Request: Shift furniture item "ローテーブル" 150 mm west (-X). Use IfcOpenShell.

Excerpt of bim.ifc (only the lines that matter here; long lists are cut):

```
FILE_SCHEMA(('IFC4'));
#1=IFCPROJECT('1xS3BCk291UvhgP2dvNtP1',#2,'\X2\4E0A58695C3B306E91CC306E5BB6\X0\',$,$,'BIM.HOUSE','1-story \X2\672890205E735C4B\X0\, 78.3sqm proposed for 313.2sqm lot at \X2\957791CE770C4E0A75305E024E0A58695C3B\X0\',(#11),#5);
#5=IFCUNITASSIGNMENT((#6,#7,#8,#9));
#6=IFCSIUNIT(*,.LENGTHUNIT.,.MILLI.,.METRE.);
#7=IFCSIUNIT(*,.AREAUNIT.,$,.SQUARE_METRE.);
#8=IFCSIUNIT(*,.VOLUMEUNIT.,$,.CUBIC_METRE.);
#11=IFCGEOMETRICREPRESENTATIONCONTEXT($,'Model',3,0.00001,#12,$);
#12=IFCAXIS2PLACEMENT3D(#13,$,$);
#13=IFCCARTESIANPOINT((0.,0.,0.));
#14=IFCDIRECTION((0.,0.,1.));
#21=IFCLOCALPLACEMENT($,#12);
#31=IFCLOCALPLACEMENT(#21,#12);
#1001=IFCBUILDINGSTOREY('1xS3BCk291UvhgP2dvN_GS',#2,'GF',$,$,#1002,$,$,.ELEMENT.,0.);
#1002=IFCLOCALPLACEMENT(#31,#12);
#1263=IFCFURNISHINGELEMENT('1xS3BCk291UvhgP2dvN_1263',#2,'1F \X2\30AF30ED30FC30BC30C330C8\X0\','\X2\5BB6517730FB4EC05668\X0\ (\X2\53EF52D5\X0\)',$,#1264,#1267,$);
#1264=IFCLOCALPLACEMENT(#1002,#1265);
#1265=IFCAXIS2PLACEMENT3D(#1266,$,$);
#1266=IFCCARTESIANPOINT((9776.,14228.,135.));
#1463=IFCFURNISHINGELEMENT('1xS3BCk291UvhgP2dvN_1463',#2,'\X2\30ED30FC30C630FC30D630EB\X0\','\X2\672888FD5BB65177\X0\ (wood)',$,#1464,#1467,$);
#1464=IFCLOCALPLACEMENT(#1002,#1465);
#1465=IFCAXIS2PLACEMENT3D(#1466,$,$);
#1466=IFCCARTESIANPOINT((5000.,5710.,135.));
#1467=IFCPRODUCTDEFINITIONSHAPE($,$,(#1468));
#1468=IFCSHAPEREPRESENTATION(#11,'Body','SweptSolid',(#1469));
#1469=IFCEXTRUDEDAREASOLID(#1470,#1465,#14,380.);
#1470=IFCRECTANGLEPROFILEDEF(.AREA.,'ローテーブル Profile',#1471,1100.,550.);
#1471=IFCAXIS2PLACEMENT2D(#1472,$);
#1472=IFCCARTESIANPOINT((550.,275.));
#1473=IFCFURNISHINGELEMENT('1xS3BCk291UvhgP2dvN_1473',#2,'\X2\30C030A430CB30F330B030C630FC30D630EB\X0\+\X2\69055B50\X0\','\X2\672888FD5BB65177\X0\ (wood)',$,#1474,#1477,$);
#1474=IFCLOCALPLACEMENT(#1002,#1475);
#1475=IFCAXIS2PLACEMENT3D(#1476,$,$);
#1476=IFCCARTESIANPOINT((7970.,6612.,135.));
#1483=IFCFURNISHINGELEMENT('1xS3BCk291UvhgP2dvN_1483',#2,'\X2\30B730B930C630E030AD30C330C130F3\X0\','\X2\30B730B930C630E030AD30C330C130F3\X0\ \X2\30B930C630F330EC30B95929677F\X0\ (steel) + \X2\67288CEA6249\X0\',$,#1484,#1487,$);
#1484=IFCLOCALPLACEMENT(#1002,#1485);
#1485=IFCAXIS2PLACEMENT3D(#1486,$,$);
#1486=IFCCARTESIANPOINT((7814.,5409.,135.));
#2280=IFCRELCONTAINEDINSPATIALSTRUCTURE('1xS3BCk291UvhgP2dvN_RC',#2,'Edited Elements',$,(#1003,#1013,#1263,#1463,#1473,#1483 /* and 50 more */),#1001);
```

```python
import ifcopenshell
import ifcopenshell.api.geometry
import ifcopenshell.util.placement
import ifcopenshell.util.unit

model = ifcopenshell.open("bim.ifc")
unit_scale = ifcopenshell.util.unit.calculate_unit_scale(model)

item = model.by_id(1463)
matrix = ifcopenshell.util.placement.get_local_placement(item.ObjectPlacement)
matrix[0, 3] -= 0.15 / unit_scale
ifcopenshell.api.geometry.edit_object_placement(model, product=item, matrix=matrix, is_si=False)

print(ifcopenshell.util.placement.get_local_placement(item.ObjectPlacement).round(3) + 0.0)

model.write("bim_rev.ifc")
```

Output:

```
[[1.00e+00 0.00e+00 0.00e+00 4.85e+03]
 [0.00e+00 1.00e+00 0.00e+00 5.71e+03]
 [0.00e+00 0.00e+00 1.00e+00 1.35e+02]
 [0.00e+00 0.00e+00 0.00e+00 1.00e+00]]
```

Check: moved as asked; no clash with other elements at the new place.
